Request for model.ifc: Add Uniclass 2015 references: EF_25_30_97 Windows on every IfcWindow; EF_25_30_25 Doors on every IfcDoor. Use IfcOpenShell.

First a look at what the model holds.

```python
import ifcopenshell

model = ifcopenshell.open("model.ifc")
print(model.schema)
print("classifications:", [c.Name for c in model.by_type("IfcClassification")])
for ifc_class in ("IfcDoor", "IfcRoof", "IfcStair", "IfcWall", "IfcWindow"):
    print(ifc_class, len(model.by_type(ifc_class)))
```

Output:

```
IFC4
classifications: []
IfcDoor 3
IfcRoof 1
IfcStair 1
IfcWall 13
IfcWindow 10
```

```python
import ifcopenshell
import ifcopenshell.api.classification

model = ifcopenshell.open("model.ifc")

system = ifcopenshell.api.classification.add_classification(model, classification="Uniclass 2015")

codes = {
    "IfcWindow": ("EF_25_30_97", "Windows"),
    "IfcDoor": ("EF_25_30_25", "Doors"),
}
for ifc_class, (code, name) in codes.items():
    products = model.by_type(ifc_class)
    ifcopenshell.api.classification.add_reference(
        model, products=products, classification=system, identification=code, name=name
    )
    print(code, len(products))

model.write("model-out.ifc")
```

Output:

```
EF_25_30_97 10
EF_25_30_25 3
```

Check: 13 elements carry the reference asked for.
